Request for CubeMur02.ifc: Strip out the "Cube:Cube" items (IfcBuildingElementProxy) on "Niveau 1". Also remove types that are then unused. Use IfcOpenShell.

First a look at what the model holds.

```python
import ifcopenshell
import ifcopenshell.util.element

model = ifcopenshell.open("CubeMur02.ifc")
print(model.schema)
storey = next(s for s in model.by_type("IfcBuildingStorey") if s.Name == "Niveau 1")
proxies = [e for e in ifcopenshell.util.element.get_decomposition(storey) if e.is_a("IfcBuildingElementProxy")]
seen = {}
for e in proxies:
    element_type = ifcopenshell.util.element.get_type(e)
    name = element_type.Name if element_type not in (None, e) else None
    seen[name] = seen.get(name, 0) + 1
for name, count in sorted(seen.items(), key=str):
    print(count, "x", name)
```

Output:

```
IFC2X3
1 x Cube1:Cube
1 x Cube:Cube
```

```python
import ifcopenshell
import ifcopenshell.api.root
import ifcopenshell.util.element

model = ifcopenshell.open("CubeMur02.ifc")

storey = next(s for s in model.by_type("IfcBuildingStorey") if s.Name == "Niveau 1")
proxies = [e for e in ifcopenshell.util.element.get_decomposition(storey) if e.is_a("IfcBuildingElementProxy")]
targets = [e for e in proxies if (t := ifcopenshell.util.element.get_type(e)) not in (None, e) and t.Name == "Cube:Cube"]
types = {ifcopenshell.util.element.get_type(e) for e in targets} - {None, *targets}

for e in targets:
    ifcopenshell.api.root.remove_product(model, product=e)
print(len(targets), "removed")

unused = [t for t in types if not ifcopenshell.util.element.get_types(t)]
for t in unused:
    ifcopenshell.api.root.remove_product(model, product=t)
print(len(unused), "unused types removed")

model.write("CubeMur02_updated.ifc")
```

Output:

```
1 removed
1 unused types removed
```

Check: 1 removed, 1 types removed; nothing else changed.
